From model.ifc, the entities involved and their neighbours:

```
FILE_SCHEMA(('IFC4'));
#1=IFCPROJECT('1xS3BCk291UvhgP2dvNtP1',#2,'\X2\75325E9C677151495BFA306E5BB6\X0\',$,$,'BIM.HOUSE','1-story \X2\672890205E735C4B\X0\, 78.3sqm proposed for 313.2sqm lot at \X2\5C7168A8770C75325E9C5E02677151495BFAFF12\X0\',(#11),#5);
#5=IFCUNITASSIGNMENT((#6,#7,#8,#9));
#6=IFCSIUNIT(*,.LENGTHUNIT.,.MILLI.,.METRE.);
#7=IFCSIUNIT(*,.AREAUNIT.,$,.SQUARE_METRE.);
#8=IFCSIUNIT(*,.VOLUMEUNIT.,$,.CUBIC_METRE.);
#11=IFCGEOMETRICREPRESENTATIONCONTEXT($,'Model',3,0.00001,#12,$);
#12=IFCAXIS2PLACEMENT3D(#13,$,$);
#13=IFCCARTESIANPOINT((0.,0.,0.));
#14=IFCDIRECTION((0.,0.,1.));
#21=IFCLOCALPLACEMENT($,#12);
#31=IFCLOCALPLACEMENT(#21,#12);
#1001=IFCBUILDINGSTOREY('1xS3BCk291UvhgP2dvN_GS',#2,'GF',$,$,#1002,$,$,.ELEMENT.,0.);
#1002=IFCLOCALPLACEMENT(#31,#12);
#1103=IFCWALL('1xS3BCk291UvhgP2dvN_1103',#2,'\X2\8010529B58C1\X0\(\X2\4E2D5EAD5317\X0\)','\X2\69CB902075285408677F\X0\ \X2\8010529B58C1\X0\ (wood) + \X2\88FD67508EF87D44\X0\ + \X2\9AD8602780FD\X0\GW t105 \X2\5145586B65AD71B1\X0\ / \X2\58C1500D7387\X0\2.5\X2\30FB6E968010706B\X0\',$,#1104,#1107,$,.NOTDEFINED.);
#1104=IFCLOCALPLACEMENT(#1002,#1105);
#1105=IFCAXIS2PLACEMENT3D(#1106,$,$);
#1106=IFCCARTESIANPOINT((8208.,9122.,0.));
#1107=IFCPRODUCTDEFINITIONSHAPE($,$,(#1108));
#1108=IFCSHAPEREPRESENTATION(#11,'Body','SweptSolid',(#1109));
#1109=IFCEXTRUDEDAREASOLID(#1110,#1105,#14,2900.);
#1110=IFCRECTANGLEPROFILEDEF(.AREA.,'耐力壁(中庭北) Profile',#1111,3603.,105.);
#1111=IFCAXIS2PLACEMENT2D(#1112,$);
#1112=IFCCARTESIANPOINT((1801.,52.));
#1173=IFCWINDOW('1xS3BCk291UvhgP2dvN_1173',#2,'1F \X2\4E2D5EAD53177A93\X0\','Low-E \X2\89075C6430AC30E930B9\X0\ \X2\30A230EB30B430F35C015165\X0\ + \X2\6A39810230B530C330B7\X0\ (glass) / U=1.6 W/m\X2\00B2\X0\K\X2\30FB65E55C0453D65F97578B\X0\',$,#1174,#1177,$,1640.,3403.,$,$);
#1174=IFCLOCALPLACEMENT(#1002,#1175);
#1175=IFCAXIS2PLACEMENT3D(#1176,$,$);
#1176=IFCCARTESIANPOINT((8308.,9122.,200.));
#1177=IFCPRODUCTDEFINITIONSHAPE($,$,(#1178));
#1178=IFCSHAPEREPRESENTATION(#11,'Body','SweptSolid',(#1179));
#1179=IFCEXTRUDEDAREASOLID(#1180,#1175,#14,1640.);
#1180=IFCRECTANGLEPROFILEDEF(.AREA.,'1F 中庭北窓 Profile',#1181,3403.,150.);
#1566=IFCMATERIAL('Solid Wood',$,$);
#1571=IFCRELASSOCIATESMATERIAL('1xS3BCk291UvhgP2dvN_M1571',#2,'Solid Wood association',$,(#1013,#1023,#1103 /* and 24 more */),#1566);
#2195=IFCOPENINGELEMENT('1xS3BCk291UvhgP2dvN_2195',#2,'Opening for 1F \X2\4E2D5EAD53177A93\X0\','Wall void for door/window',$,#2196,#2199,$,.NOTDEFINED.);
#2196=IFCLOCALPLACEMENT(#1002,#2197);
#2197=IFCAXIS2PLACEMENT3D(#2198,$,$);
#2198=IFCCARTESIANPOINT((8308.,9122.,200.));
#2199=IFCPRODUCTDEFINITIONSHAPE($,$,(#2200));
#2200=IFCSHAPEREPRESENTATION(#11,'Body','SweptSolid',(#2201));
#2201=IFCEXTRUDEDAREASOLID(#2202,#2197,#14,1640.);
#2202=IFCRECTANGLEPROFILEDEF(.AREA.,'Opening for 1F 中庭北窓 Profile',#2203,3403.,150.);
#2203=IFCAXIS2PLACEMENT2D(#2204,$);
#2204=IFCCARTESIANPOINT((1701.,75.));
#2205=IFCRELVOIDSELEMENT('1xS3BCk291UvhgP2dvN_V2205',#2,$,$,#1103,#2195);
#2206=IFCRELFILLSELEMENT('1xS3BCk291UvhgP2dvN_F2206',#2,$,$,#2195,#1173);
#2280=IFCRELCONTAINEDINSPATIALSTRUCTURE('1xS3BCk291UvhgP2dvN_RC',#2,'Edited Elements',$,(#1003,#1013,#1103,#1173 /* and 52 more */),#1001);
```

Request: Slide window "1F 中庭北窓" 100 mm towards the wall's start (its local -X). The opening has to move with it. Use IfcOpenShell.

```python
import ifcopenshell
import ifcopenshell.api.geometry
import ifcopenshell.util.placement
import ifcopenshell.util.unit

model = ifcopenshell.open("model.ifc")
unit_scale = ifcopenshell.util.unit.calculate_unit_scale(model)

window = model.by_id(1173)
opening = window.FillsVoids[0].RelatingOpeningElement
wall = opening.VoidsElements[0].RelatingBuildingElement

wall_matrix = ifcopenshell.util.placement.get_local_placement(wall.ObjectPlacement)
shift = wall_matrix[:3, 0] * -0.1 / unit_scale
before = ifcopenshell.util.placement.get_local_placement(window.ObjectPlacement)[:3, 3].copy()

# The window is not placed relative to its opening, so move both.
for product in (opening, window):
    matrix = ifcopenshell.util.placement.get_local_placement(product.ObjectPlacement)
    matrix[:3, 3] += shift
    ifcopenshell.api.geometry.edit_object_placement(model, product=product, matrix=matrix, is_si=False)

after = ifcopenshell.util.placement.get_local_placement(window.ObjectPlacement)[:3, 3]
print("window moved by", (after - before).round(3) + 0.0)

model.write("model_v2.ifc")
```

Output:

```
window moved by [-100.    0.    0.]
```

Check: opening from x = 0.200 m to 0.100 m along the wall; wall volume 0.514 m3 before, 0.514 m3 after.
